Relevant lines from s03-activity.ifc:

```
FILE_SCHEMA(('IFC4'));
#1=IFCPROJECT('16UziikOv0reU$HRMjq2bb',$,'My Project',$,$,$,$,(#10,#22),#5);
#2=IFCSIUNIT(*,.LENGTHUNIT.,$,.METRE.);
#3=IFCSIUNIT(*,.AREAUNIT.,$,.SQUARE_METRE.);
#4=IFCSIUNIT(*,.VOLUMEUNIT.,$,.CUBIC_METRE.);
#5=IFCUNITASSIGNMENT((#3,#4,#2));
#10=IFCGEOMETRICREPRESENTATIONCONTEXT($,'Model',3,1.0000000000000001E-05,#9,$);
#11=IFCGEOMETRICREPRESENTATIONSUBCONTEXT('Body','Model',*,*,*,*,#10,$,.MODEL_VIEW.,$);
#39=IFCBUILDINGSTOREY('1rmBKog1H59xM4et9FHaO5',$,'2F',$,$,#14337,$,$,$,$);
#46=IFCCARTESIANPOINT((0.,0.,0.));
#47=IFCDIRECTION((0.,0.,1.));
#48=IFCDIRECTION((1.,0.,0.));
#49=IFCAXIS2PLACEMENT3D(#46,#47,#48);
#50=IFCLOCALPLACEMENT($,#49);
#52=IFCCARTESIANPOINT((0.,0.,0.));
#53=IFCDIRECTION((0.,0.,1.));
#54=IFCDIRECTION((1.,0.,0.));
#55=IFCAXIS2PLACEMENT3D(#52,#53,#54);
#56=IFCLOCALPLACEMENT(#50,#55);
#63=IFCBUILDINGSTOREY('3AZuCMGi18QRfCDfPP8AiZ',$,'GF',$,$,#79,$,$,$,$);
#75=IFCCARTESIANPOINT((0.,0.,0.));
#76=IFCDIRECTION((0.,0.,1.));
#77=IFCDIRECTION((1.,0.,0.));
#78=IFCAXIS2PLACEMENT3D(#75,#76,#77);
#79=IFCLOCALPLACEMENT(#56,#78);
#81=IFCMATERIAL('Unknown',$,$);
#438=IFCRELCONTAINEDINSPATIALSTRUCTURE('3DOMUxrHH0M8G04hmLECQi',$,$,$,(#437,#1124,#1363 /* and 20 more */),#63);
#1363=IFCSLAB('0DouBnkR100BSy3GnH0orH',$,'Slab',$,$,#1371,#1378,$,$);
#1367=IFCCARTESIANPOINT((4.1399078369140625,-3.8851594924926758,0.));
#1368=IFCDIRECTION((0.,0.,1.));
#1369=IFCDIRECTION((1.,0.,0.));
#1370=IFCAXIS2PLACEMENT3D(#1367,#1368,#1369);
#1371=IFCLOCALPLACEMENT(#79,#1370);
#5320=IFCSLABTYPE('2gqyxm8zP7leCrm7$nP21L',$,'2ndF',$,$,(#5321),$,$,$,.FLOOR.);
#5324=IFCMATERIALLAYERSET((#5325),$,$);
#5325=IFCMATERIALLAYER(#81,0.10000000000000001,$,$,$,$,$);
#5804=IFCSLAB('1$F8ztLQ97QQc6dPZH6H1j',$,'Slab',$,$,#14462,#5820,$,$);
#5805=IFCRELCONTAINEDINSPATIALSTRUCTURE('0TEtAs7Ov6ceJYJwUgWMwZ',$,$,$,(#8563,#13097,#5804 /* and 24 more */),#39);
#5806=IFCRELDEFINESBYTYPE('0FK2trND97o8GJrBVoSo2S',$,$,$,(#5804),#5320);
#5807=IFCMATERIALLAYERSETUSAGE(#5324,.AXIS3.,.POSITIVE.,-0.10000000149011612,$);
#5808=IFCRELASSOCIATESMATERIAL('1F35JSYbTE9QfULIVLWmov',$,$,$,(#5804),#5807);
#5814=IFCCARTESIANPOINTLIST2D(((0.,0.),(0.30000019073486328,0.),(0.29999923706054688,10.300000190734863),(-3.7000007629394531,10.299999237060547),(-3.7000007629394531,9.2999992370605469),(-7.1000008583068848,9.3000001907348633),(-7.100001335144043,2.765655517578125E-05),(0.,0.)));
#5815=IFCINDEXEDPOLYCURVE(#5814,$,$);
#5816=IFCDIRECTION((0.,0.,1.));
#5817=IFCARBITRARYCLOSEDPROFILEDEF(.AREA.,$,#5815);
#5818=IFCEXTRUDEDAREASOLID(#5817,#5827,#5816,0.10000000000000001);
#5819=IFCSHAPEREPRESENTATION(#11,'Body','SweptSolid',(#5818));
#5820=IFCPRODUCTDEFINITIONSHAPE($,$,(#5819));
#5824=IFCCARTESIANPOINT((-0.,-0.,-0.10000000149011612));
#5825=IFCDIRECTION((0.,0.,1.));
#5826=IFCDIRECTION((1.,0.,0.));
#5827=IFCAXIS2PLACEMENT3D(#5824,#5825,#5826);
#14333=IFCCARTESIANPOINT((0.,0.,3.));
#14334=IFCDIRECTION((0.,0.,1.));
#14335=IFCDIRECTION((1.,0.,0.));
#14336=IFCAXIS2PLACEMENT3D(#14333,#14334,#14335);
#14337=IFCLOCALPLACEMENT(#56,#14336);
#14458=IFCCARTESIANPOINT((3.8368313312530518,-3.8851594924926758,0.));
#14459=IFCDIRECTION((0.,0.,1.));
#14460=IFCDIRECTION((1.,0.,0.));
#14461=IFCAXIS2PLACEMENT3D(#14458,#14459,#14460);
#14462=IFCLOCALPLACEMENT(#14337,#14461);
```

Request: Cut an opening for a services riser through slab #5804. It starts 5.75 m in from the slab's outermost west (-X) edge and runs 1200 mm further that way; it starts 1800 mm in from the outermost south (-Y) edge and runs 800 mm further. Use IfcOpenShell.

```python
import numpy as np
import ifcopenshell
import ifcopenshell.api.feature
import ifcopenshell.api.geometry
import ifcopenshell.api.root
import ifcopenshell.geom
import ifcopenshell.util.placement
import ifcopenshell.util.representation
import ifcopenshell.util.shape
import ifcopenshell.util.unit

model = ifcopenshell.open("s03-activity.ifc")
unit_scale = ifcopenshell.util.unit.calculate_unit_scale(model)
settings = ifcopenshell.geom.settings()


def volume(element):
    """Net volume in cubic metres, openings subtracted."""
    shape = ifcopenshell.geom.create_shape(settings, element)
    return ifcopenshell.util.shape.get_volume(shape.geometry)


slab = model.by_guid("1$F8ztLQ97QQc6dPZH6H1j")
before = volume(slab)

# Extent in the slab's own axes, in metres. The edges named are its -X and -Y sides.
slab_shape = ifcopenshell.geom.create_shape(settings, slab)
vertices = ifcopenshell.util.shape.get_vertices(slab_shape.geometry)
x_min, y_min, bottom = vertices.min(axis=0)
top = vertices[:, 2].max()

opening = ifcopenshell.api.root.create_entity(model, ifc_class="IfcOpeningElement", name="Services riser opening", predefined_type="OPENING")
context = ifcopenshell.util.representation.get_context(model, "Model", "Body", "MODEL_VIEW")
width, depth = 1.2, 0.8
outline = [(0.0, 0.0), (width, 0.0), (width, depth), (0.0, depth), (0.0, 0.0)]
# Overshoot both faces by 50 mm so the cut is clean.
shape = ifcopenshell.api.geometry.add_slab_representation(
    model, context=context, depth=top - bottom + 0.1, polyline=outline
)
ifcopenshell.api.geometry.assign_representation(model, product=opening, representation=shape)

matrix = ifcopenshell.util.placement.get_local_placement(slab.ObjectPlacement)
matrix[:, 3] = matrix @ np.append(np.array([x_min + 5.75, y_min + 1.8, bottom - 0.05]) / unit_scale, 1.0)
ifcopenshell.api.geometry.edit_object_placement(model, product=opening, matrix=matrix, is_si=False)
ifcopenshell.api.feature.add_feature(model, feature=opening, element=slab)

after = volume(slab)

print(f"slab volume {before:.3f} -> {after:.3f} m3")

model.write("s03-activity_rev.ifc")
```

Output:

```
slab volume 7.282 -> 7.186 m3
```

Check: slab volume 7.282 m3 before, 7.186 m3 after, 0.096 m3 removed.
